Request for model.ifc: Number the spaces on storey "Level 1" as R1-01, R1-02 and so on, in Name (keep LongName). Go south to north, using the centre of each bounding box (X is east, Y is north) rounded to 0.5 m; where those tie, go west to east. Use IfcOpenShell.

First a look at what the model holds.

```python
import ifcopenshell
import ifcopenshell.util.element
import ifcopenshell.util.placement

model = ifcopenshell.open("model.ifc")
print(model.schema)
storey = next(s for s in model.by_type("IfcBuildingStorey") if s.Name == "Level 1")
spaces = [e for e in ifcopenshell.util.element.get_decomposition(storey) if e.is_a("IfcSpace")]
for e in sorted(spaces, key=lambda e: e.id()):
    origin = ifcopenshell.util.placement.get_local_placement(e.ObjectPlacement)[:3, 3]
    print(e.id(), e.Name, e.LongName, origin.round(2) + 0.0, sep=" | ")
```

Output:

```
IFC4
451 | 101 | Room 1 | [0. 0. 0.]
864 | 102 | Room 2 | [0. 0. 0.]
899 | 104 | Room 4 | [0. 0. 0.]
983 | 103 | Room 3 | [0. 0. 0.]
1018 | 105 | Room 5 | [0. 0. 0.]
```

```python
import ifcopenshell
import ifcopenshell.geom
import ifcopenshell.util.element
import ifcopenshell.util.shape

model = ifcopenshell.open("model.ifc")
settings = ifcopenshell.geom.settings()
settings.set("use-world-coords", True)


def centre(element):
    shape = ifcopenshell.geom.create_shape(settings, element)
    return ifcopenshell.util.shape.get_bbox_centroid(shape.geometry)


storey = next(s for s in model.by_type("IfcBuildingStorey") if s.Name == "Level 1")
spaces = [e for e in ifcopenshell.util.element.get_decomposition(storey) if e.is_a("IfcSpace")]

# Insertion points can sit at a corner or the storey origin, so sort by the geometry (in metres).
centres = {e: centre(e) for e in spaces}
spaces.sort(key=lambda e: (round(centres[e][1] / 0.5), centres[e][0]))

for i, e in enumerate(spaces, start=1):
    number = f"R1-{i:02d}"
    e.Name = number
    print(e.id(), number)

model.write("model_v2.ifc")
```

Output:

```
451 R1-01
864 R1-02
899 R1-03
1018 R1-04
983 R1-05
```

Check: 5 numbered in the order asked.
